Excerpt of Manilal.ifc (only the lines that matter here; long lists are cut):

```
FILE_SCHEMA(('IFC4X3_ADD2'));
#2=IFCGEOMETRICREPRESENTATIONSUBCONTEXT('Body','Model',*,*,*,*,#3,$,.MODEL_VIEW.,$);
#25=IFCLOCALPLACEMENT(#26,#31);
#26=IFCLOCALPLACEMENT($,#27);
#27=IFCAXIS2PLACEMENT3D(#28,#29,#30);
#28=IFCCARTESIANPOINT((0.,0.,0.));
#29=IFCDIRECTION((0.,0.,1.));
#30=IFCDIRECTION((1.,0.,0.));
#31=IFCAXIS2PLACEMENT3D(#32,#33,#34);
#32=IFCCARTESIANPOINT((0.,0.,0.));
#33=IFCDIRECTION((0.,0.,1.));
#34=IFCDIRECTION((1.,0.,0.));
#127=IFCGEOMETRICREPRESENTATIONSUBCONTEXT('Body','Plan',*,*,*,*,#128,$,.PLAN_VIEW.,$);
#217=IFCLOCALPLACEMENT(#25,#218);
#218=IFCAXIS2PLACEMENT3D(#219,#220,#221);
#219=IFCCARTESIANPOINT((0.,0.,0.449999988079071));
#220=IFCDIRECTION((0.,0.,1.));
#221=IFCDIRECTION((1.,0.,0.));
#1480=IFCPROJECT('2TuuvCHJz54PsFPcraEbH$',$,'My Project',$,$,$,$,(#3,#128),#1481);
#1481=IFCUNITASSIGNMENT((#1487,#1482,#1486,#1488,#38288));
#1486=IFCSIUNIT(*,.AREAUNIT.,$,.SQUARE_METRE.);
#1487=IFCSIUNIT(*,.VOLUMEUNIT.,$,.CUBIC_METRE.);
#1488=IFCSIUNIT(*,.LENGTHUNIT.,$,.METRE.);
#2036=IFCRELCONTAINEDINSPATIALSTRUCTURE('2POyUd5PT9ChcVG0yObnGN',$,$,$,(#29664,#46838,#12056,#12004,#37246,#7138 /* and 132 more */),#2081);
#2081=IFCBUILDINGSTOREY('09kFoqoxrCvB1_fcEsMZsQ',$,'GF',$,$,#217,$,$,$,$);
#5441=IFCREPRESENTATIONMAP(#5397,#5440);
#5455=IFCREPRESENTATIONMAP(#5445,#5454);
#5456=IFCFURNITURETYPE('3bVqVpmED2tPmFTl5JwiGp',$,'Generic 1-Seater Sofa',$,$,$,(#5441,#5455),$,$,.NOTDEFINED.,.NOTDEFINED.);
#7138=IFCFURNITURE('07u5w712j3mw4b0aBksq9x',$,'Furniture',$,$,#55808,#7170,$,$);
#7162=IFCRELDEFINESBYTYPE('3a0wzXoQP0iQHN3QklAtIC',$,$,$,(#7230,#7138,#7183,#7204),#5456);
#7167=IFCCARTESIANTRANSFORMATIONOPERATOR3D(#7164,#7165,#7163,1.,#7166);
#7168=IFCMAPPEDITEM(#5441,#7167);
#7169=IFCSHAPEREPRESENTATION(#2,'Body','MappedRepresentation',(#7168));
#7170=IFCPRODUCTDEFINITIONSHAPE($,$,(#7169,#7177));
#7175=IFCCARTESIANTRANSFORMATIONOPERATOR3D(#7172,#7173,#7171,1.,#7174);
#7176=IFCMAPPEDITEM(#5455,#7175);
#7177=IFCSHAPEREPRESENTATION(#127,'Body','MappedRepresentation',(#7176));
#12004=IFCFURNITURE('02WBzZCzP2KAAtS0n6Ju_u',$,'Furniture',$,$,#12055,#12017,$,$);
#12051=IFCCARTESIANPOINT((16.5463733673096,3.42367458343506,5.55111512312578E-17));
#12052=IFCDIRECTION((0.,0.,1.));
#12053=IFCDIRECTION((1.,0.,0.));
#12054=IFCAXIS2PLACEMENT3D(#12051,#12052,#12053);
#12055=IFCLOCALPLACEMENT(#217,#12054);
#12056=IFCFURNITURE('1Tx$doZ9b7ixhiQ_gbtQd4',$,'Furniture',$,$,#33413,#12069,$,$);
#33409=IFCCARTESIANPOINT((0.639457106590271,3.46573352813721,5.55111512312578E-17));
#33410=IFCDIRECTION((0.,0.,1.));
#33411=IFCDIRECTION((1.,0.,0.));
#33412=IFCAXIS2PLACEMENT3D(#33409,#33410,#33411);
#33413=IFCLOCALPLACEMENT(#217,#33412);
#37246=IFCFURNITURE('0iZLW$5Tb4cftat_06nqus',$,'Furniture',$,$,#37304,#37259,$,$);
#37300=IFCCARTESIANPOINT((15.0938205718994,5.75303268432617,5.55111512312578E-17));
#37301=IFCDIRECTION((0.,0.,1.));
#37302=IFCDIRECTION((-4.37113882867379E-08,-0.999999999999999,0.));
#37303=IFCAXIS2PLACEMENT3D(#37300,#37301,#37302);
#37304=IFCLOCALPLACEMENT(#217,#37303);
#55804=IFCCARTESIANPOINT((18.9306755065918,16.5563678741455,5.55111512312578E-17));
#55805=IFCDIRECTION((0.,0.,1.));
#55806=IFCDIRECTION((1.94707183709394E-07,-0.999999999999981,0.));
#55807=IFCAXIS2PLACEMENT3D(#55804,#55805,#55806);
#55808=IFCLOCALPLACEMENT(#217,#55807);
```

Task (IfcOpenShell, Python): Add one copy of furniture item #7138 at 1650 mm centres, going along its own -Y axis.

```python
import ifcopenshell
import ifcopenshell.api.geometry
import ifcopenshell.api.root
import ifcopenshell.util.element
import ifcopenshell.util.placement
import ifcopenshell.util.unit

model = ifcopenshell.open("Manilal.ifc")
unit_scale = ifcopenshell.util.unit.calculate_unit_scale(model)

source = model.by_guid("07u5w712j3mw4b0aBksq9x")
base = ifcopenshell.util.placement.get_local_placement(source.ObjectPlacement)
step = -base[:3, 1] * 1.65 / unit_scale

for i in range(1, 2):
    copy = ifcopenshell.api.root.copy_class(model, product=source)
    copy.Representation = ifcopenshell.util.element.copy_deep(
        model, source.Representation, exclude=["IfcGeometricRepresentationContext", "IfcRepresentationMap"]
    )
    matrix = base.copy()
    matrix[:3, 3] += i * step
    print("added at", matrix[:3, 3].round(3) + 0.0)
    ifcopenshell.api.geometry.edit_object_placement(model, product=copy, matrix=matrix, is_si=False)

model.write("Manilal_rev.ifc")
```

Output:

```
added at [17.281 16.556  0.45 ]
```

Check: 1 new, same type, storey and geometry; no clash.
